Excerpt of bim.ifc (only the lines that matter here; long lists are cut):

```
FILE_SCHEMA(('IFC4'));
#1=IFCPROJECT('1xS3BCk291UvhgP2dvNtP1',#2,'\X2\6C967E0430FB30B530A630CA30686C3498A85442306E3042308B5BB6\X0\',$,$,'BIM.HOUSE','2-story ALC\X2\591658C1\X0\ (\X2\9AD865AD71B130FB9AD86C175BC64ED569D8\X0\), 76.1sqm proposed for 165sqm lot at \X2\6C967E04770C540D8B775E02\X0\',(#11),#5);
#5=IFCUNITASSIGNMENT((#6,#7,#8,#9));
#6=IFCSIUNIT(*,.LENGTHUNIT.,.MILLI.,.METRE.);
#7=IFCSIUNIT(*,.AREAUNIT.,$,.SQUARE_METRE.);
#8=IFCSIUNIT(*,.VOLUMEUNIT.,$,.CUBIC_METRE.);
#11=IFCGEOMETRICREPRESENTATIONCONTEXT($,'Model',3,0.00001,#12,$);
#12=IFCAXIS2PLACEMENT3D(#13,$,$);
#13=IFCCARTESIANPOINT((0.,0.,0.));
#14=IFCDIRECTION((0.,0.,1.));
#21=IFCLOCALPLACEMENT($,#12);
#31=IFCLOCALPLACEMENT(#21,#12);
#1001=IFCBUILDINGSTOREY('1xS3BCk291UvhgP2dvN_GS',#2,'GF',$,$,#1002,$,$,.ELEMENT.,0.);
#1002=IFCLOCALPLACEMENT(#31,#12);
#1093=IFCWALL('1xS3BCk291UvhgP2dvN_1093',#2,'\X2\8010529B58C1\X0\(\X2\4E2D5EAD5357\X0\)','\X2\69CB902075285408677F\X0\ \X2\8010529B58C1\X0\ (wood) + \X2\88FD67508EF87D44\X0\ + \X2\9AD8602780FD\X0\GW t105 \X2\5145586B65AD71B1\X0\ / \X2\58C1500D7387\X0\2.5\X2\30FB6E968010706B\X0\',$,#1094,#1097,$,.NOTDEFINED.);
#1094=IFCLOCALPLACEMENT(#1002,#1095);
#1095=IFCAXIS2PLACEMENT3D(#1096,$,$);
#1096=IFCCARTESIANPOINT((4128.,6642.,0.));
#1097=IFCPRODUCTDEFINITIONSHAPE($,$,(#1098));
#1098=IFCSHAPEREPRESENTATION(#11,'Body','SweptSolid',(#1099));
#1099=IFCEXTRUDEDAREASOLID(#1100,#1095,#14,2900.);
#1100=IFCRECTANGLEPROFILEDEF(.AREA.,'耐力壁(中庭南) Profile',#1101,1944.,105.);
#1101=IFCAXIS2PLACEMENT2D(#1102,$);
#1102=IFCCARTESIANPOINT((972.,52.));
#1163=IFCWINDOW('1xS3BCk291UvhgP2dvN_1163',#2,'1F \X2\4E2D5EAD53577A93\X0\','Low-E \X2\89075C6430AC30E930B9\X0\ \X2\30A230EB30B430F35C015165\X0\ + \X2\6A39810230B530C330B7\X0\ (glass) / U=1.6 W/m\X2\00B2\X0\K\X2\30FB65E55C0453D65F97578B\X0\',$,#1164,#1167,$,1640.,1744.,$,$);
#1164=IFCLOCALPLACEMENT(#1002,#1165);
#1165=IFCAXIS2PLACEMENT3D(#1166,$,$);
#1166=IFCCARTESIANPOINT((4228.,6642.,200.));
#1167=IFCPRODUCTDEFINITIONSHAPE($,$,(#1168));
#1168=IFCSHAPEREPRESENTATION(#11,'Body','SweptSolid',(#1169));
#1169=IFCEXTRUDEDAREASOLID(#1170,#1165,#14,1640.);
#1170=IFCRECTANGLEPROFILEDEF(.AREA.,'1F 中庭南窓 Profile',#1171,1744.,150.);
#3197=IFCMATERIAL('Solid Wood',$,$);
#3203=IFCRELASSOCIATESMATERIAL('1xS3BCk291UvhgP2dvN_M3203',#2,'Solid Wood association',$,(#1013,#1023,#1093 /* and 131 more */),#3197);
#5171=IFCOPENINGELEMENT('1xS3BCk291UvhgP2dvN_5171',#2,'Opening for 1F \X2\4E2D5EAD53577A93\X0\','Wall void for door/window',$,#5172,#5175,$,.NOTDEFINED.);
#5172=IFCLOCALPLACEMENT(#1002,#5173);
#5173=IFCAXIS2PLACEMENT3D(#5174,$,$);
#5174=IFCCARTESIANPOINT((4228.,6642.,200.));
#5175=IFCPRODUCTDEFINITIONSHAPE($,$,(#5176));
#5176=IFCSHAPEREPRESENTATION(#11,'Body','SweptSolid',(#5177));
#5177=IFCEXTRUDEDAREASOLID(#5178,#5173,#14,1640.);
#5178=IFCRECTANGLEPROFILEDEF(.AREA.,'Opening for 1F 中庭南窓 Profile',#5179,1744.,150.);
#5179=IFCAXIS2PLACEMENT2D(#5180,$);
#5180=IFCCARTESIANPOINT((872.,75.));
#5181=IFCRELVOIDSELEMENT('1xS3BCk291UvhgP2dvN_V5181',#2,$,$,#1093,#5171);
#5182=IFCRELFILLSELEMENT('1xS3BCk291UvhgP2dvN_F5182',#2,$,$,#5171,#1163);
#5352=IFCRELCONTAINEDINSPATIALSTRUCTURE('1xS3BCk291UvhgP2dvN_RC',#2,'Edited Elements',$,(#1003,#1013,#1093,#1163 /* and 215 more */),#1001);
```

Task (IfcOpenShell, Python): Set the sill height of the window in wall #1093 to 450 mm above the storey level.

```python
import numpy as np
import ifcopenshell
import ifcopenshell.api.geometry
import ifcopenshell.geom
import ifcopenshell.util.element
import ifcopenshell.util.placement
import ifcopenshell.util.shape
import ifcopenshell.util.unit

model = ifcopenshell.open("bim.ifc")
unit_scale = ifcopenshell.util.unit.calculate_unit_scale(model)

window = model.by_guid("1xS3BCk291UvhgP2dvN_1163")
opening = window.FillsVoids[0].RelatingOpeningElement
storey = ifcopenshell.util.element.get_container(window, ifc_class="IfcBuildingStorey")
level = ifcopenshell.util.placement.get_local_placement(storey.ObjectPlacement)[2, 3]

# The opening's origin need not be at the sill, so measure its lowest point.
shape = ifcopenshell.geom.create_shape(ifcopenshell.geom.settings(), opening)
bottom = ifcopenshell.util.shape.get_shape_bottom_elevation(shape, shape.geometry) / unit_scale
dz = level + 450.0 - bottom

shift = np.array([0.0, 0.0, dz])
# The window is not placed relative to its opening, so move both.
for product in (opening, window):
    matrix = ifcopenshell.util.placement.get_local_placement(product.ObjectPlacement)
    matrix[:3, 3] += shift
    ifcopenshell.api.geometry.edit_object_placement(model, product=product, matrix=matrix, is_si=False)

print(f"moved by {dz * unit_scale:+.3f} m")

model.write("bim-out.ifc")
```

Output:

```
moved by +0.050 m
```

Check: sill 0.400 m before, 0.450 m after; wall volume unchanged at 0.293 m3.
